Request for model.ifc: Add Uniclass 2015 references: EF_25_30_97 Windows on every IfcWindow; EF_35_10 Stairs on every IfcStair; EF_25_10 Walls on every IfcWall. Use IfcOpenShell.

First a look at what the model holds.

```python
import ifcopenshell

model = ifcopenshell.open("model.ifc")
print(model.schema)
print("classifications:", [c.Name for c in model.by_type("IfcClassification")])
for ifc_class in ("IfcDoor", "IfcRoof", "IfcStair", "IfcWall", "IfcWindow"):
    print(ifc_class, len(model.by_type(ifc_class)))
```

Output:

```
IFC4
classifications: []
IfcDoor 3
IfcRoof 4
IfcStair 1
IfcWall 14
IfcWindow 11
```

```python
import ifcopenshell
import ifcopenshell.api.classification

model = ifcopenshell.open("model.ifc")

system = ifcopenshell.api.classification.add_classification(model, classification="Uniclass 2015")

codes = {
    "IfcWindow": ("EF_25_30_97", "Windows"),
    "IfcStair": ("EF_35_10", "Stairs"),
    "IfcWall": ("EF_25_10", "Walls"),
}
for ifc_class, (code, name) in codes.items():
    products = model.by_type(ifc_class)
    ifcopenshell.api.classification.add_reference(
        model, products=products, classification=system, identification=code, name=name
    )
    print(code, len(products))

model.write("model_v2.ifc")
```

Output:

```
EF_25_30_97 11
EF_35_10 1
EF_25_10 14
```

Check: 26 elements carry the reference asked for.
